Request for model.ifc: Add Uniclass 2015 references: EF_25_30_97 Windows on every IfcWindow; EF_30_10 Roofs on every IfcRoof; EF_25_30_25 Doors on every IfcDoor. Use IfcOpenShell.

First a look at what the model holds.

```python
import ifcopenshell

model = ifcopenshell.open("model.ifc")
print(model.schema)
print("classifications:", [c.Name for c in model.by_type("IfcClassification")])
for ifc_class in ("IfcDoor", "IfcRoof", "IfcStair", "IfcWall", "IfcWindow"):
    print(ifc_class, len(model.by_type(ifc_class)))
```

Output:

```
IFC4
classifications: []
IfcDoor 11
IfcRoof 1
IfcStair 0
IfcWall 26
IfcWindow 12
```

```python
import ifcopenshell
import ifcopenshell.api.classification

model = ifcopenshell.open("model.ifc")

system = ifcopenshell.api.classification.add_classification(model, classification="Uniclass 2015")

codes = {
    "IfcWindow": ("EF_25_30_97", "Windows"),
    "IfcRoof": ("EF_30_10", "Roofs"),
    "IfcDoor": ("EF_25_30_25", "Doors"),
}
for ifc_class, (code, name) in codes.items():
    products = model.by_type(ifc_class)
    ifcopenshell.api.classification.add_reference(
        model, products=products, classification=system, identification=code, name=name
    )
    print(code, len(products))

model.write("model-out.ifc")
```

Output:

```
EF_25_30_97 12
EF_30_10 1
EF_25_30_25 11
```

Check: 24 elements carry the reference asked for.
